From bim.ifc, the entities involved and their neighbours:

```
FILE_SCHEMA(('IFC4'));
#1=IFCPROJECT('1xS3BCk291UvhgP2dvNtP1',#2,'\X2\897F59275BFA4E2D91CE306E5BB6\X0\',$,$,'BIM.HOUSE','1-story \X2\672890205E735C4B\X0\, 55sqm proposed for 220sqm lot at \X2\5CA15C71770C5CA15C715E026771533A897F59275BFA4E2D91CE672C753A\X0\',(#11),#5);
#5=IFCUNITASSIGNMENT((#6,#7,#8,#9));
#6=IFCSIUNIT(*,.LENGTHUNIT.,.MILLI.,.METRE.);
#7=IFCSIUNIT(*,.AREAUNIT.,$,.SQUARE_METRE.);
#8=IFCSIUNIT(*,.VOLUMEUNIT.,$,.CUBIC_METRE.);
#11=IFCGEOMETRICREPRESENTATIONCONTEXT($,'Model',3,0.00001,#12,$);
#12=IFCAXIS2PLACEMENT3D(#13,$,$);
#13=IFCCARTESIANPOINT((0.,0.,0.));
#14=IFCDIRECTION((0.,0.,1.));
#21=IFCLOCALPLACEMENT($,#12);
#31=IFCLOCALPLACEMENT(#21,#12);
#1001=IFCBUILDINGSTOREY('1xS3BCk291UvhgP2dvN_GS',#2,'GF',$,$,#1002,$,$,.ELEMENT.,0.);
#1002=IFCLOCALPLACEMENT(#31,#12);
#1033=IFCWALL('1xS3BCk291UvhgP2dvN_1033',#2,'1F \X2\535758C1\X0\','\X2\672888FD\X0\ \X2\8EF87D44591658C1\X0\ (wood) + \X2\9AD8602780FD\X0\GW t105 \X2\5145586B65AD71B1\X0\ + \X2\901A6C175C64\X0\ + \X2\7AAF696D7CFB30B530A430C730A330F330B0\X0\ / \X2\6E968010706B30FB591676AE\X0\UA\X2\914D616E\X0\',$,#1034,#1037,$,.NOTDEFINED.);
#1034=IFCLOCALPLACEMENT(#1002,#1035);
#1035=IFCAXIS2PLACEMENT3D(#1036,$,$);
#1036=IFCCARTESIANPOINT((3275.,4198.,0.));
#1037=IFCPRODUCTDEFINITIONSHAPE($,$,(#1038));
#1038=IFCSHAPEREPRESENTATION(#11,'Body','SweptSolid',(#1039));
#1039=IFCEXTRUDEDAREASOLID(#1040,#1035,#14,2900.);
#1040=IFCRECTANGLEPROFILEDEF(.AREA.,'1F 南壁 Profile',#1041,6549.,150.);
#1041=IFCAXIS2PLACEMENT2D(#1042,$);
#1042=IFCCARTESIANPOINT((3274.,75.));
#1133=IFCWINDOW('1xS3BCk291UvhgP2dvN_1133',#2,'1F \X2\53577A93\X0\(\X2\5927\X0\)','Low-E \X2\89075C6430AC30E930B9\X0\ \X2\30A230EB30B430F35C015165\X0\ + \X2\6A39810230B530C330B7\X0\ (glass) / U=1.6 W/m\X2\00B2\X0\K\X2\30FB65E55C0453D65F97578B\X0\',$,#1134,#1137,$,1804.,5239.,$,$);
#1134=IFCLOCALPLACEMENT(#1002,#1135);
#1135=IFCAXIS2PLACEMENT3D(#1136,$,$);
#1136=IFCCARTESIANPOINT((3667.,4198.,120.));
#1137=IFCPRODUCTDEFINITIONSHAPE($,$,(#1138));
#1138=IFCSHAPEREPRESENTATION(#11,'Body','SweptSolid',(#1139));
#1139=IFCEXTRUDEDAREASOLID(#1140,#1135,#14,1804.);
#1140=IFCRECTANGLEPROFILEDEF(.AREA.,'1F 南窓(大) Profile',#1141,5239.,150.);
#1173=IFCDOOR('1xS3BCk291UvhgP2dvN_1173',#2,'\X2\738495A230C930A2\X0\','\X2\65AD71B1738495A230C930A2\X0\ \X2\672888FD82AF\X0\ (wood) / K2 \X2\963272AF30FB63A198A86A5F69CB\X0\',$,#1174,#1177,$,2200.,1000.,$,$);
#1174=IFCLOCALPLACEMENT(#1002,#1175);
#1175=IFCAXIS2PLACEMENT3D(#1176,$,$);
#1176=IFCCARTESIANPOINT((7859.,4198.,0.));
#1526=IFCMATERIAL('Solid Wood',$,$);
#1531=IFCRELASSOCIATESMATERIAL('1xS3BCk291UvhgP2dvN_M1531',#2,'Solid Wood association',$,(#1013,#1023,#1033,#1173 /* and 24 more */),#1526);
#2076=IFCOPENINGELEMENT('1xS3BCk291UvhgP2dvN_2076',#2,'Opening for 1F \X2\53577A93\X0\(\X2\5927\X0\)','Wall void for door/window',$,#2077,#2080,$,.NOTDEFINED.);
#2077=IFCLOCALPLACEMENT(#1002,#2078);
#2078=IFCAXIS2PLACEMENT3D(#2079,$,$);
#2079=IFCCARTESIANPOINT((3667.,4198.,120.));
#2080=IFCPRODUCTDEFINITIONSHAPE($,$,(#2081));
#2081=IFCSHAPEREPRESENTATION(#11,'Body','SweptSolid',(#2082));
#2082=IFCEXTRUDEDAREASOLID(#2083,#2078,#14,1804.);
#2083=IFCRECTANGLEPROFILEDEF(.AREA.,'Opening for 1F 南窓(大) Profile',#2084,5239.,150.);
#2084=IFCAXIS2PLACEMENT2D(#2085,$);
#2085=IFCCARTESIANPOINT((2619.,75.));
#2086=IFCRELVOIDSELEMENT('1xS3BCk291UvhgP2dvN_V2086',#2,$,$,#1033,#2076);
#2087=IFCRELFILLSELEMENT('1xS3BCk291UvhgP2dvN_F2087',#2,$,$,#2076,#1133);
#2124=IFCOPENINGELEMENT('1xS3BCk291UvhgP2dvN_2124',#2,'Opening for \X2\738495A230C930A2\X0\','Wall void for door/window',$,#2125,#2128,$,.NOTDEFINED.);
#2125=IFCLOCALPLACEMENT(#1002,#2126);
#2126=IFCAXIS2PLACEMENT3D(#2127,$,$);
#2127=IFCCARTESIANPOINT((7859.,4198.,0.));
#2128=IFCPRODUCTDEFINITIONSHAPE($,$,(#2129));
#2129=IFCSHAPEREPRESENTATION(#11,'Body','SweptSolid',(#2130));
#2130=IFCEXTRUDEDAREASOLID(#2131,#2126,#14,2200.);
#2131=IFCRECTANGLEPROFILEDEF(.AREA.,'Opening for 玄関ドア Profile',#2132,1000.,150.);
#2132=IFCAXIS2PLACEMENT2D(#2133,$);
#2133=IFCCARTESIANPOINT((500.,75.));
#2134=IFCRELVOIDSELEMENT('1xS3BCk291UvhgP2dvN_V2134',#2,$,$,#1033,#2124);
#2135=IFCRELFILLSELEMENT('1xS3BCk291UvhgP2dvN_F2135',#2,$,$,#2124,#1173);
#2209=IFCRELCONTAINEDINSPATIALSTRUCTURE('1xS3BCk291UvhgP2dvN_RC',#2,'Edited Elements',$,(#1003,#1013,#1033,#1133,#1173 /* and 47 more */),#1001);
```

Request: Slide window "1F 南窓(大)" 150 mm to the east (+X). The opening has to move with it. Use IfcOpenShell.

```python
import ifcopenshell
import ifcopenshell.api.geometry
import ifcopenshell.util.placement

model = ifcopenshell.open("bim.ifc")

window = model.by_guid("1xS3BCk291UvhgP2dvN_1133")
opening = window.FillsVoids[0].RelatingOpeningElement
wall = opening.VoidsElements[0].RelatingBuildingElement

wall_matrix = ifcopenshell.util.placement.get_local_placement(wall.ObjectPlacement)
shift = wall_matrix[:3, 0] * 150.0
before = ifcopenshell.util.placement.get_local_placement(window.ObjectPlacement)[:3, 3].copy()

# The window is not placed relative to its opening, so move both.
for product in (opening, window):
    matrix = ifcopenshell.util.placement.get_local_placement(product.ObjectPlacement)
    matrix[:3, 3] += shift
    ifcopenshell.api.geometry.edit_object_placement(model, product=product, matrix=matrix, is_si=False)

after = ifcopenshell.util.placement.get_local_placement(window.ObjectPlacement)[:3, 3]
print("window moved by", (after - before).round(3) + 0.0)

model.write("bim-out.ifc")
```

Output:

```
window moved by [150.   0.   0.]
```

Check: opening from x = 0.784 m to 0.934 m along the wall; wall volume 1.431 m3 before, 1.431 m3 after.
